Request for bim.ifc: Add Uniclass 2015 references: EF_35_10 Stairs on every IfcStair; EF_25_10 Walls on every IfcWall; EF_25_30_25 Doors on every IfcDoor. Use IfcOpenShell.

First a look at what the model holds.

```python
import ifcopenshell

model = ifcopenshell.open("bim.ifc")
print(model.schema)
print("classifications:", [c.Name for c in model.by_type("IfcClassification")])
for ifc_class in ("IfcDoor", "IfcRoof", "IfcStair", "IfcWall", "IfcWindow"):
    print(ifc_class, len(model.by_type(ifc_class)))
```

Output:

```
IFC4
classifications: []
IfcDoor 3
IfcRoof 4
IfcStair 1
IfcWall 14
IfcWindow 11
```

```python
import ifcopenshell
import ifcopenshell.api.classification

model = ifcopenshell.open("bim.ifc")

system = ifcopenshell.api.classification.add_classification(model, classification="Uniclass 2015")

codes = {
    "IfcStair": ("EF_35_10", "Stairs"),
    "IfcWall": ("EF_25_10", "Walls"),
    "IfcDoor": ("EF_25_30_25", "Doors"),
}
for ifc_class, (code, name) in codes.items():
    products = model.by_type(ifc_class)
    ifcopenshell.api.classification.add_reference(
        model, products=products, classification=system, identification=code, name=name
    )
    print(code, len(products))

model.write("bim_rev.ifc")
```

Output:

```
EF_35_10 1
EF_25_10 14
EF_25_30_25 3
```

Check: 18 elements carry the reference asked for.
